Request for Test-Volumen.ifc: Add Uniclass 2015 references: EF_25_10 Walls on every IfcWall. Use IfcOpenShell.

First a look at what the model holds.

```python
import ifcopenshell

model = ifcopenshell.open("Test-Volumen.ifc")
print(model.schema)
print("classifications:", [c.Name for c in model.by_type("IfcClassification")])
for ifc_class in ("IfcDoor", "IfcRoof", "IfcStair", "IfcWall", "IfcWindow"):
    print(ifc_class, len(model.by_type(ifc_class)))
```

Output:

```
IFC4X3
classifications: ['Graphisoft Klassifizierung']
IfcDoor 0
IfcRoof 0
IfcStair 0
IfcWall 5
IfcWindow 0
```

```python
import ifcopenshell
import ifcopenshell.api.classification

model = ifcopenshell.open("Test-Volumen.ifc")

system = ifcopenshell.api.classification.add_classification(model, classification="Uniclass 2015")

codes = {
    "IfcWall": ("EF_25_10", "Walls"),
}
for ifc_class, (code, name) in codes.items():
    products = model.by_type(ifc_class)
    ifcopenshell.api.classification.add_reference(
        model, products=products, classification=system, identification=code, name=name
    )
    print(code, len(products))

model.write("Test-Volumen_edited.ifc")
```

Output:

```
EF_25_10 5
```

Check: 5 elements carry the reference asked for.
